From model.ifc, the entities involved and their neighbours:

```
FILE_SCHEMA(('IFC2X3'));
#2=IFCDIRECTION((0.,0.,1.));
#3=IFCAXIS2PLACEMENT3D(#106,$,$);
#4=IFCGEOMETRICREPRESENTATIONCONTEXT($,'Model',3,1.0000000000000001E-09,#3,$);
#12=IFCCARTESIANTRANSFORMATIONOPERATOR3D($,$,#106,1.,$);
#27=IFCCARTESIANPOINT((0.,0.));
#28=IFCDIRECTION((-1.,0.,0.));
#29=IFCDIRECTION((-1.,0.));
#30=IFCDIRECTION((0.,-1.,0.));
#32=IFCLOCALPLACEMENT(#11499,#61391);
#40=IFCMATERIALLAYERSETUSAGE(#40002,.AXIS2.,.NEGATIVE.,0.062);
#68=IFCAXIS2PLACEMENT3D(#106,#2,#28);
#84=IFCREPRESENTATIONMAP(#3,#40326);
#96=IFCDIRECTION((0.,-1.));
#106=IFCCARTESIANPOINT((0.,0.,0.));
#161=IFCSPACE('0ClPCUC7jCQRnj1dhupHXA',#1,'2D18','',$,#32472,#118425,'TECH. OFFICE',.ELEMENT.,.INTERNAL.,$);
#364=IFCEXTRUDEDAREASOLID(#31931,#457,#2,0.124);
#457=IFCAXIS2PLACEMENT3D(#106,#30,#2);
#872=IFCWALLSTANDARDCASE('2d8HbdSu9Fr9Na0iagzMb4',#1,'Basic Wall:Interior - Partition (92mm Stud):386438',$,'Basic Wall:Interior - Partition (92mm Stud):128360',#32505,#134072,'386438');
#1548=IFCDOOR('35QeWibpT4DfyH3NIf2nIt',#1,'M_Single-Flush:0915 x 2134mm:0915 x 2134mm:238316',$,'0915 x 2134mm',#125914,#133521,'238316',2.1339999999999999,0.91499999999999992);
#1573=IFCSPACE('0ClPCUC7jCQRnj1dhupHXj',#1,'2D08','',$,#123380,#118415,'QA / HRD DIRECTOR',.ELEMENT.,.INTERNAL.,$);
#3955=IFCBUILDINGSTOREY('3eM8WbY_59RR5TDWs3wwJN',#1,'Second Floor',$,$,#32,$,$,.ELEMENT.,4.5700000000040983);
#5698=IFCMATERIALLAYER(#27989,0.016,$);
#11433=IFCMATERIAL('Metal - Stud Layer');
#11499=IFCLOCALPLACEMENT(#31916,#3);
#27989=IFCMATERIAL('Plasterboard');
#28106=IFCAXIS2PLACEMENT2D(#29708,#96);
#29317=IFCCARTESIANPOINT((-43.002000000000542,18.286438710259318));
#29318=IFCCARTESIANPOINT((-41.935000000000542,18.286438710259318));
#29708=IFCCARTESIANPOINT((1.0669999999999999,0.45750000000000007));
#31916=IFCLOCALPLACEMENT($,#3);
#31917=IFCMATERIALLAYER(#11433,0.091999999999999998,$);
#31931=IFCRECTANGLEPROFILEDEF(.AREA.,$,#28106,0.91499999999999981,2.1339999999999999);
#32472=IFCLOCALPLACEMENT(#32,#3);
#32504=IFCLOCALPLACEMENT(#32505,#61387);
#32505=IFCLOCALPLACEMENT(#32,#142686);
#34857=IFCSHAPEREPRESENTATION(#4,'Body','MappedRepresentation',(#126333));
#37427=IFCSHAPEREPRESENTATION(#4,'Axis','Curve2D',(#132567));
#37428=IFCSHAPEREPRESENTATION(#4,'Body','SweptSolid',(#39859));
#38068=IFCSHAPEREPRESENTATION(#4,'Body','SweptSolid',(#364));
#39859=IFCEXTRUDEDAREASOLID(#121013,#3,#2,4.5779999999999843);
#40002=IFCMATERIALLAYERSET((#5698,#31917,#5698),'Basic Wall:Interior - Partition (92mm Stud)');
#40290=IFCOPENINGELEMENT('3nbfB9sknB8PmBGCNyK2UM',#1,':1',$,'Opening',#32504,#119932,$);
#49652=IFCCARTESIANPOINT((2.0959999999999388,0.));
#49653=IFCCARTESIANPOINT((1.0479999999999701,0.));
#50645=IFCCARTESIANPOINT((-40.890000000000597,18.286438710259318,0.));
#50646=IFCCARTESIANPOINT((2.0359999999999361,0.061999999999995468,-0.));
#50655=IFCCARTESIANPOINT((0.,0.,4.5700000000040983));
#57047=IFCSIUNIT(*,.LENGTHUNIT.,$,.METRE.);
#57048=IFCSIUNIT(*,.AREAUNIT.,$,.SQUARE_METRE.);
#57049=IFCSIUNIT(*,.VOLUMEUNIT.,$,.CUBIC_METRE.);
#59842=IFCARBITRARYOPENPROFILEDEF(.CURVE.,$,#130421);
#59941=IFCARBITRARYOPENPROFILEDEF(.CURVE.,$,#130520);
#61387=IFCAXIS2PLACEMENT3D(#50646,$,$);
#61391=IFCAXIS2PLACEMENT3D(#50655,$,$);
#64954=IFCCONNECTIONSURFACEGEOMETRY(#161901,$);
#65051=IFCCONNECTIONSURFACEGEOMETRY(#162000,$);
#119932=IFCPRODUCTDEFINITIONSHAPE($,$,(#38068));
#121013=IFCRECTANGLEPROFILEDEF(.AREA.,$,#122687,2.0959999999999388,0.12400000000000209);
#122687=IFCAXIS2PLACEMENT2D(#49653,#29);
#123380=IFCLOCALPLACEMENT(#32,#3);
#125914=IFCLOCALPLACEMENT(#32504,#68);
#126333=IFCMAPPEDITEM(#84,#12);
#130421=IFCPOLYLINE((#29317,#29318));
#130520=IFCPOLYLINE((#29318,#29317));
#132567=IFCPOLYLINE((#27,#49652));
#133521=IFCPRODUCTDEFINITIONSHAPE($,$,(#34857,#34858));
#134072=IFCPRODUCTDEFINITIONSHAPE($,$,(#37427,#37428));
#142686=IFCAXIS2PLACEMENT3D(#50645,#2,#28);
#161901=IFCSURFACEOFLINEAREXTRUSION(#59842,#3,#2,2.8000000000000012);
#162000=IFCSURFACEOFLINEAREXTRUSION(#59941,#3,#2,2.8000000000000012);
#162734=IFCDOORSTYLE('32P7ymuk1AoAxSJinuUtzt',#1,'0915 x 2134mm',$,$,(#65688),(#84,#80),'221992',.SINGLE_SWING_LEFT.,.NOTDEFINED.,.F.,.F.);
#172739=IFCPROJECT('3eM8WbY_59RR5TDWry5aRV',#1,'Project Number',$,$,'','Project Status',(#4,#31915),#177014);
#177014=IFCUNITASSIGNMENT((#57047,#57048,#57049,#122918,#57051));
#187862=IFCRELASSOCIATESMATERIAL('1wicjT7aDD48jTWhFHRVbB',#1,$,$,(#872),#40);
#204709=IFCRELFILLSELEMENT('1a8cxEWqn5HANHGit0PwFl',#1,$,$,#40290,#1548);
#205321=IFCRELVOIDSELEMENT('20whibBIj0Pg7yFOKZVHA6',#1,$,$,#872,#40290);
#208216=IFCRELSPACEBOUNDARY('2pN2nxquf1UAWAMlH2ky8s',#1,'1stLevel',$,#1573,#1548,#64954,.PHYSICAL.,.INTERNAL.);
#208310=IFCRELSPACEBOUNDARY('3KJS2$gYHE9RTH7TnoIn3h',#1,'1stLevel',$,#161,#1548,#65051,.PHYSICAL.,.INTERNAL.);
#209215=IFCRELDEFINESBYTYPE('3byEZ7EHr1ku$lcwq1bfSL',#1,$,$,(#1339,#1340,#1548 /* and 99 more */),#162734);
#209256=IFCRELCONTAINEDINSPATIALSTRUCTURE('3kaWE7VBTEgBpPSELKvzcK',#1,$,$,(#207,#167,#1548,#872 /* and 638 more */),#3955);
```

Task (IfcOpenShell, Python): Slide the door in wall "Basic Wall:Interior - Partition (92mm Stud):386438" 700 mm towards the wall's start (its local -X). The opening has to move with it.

```python
import numpy as np
import ifcopenshell
import ifcopenshell.api.geometry
import ifcopenshell.util.placement

model = ifcopenshell.open("model.ifc")

door = model.by_guid("35QeWibpT4DfyH3NIf2nIt")
opening = door.FillsVoids[0].RelatingOpeningElement
wall = opening.VoidsElements[0].RelatingBuildingElement

wall_matrix = ifcopenshell.util.placement.get_local_placement(wall.ObjectPlacement)
shift = wall_matrix[:3, 0] * -0.7
before = ifcopenshell.util.placement.get_local_placement(door.ObjectPlacement)[:3, 3].copy()

# The door is placed relative to its opening, so it follows when the opening moves.
matrix = ifcopenshell.util.placement.get_local_placement(opening.ObjectPlacement)
matrix[:3, 3] += shift
ifcopenshell.api.geometry.edit_object_placement(
    model, product=opening, matrix=matrix, is_si=False, should_transform_children=True
)

# Space boundary surfaces are stored in each space's coordinates; move them too.
for rel in door.ProvidesBoundaries:
    if not rel.ConnectionGeometry:
        continue
    surface = rel.ConnectionGeometry.SurfaceOnRelatingElement
    space_matrix = ifcopenshell.util.placement.get_local_placement(rel.RelatingSpace.ObjectPlacement)
    point = np.array(surface.Position.Location.Coordinates) + space_matrix[:3, :3].T @ shift
    surface.Position = model.createIfcAxis2Placement3D(
        model.createIfcCartesianPoint(point.tolist()), surface.Position.Axis, surface.Position.RefDirection
    )

after = ifcopenshell.util.placement.get_local_placement(door.ObjectPlacement)[:3, 3]
print("door moved by", (after - before).round(3) + 0.0)

model.write("model-out.ifc")
```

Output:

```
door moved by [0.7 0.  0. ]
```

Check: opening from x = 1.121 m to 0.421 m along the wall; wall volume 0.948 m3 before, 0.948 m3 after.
